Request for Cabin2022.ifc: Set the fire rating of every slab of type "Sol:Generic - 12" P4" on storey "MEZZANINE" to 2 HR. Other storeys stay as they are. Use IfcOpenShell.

First a look at what the model holds.

```python
import ifcopenshell
import ifcopenshell.util.element

model = ifcopenshell.open("Cabin2022.ifc")
print(model.schema)
storey = next(s for s in model.by_type("IfcBuildingStorey") if s.Name == "MEZZANINE")
slabs = [e for e in ifcopenshell.util.element.get_decomposition(storey) if e.is_a("IfcSlab")]
seen = {}
for e in slabs:
    element_type = ifcopenshell.util.element.get_type(e)
    key = (element_type.Name if element_type != e and element_type else None, ifcopenshell.util.element.get_pset(e, "Pset_SlabCommon", "FireRating"))
    seen[key] = seen.get(key, 0) + 1
for (name, value), count in sorted(seen.items(), key=str):
    print(count, "x", name, "|", value)
```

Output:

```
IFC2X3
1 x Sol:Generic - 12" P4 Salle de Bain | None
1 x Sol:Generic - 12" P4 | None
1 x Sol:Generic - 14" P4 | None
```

```python
import ifcopenshell
import ifcopenshell.api.pset
import ifcopenshell.util.element

model = ifcopenshell.open("Cabin2022.ifc")

storey = next(s for s in model.by_type("IfcBuildingStorey") if s.Name == "MEZZANINE")
slabs = [e for e in ifcopenshell.util.element.get_decomposition(storey) if e.is_a("IfcSlab")]

count = 0
for e in slabs:
    element_type = ifcopenshell.util.element.get_type(e)
    if element_type in (None, e) or element_type.Name != 'Sol:Generic - 12" P4':
        continue
    # add_pset returns the element's existing set when there is one.
    pset = ifcopenshell.api.pset.add_pset(model, product=e, name="Pset_SlabCommon")
    ifcopenshell.api.pset.edit_pset(model, pset=pset, properties={"FireRating": "2 HR"})
    count += 1

print(count, "slabs updated")

model.write("Cabin2022_edited.ifc")
```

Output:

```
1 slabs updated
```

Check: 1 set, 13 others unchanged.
